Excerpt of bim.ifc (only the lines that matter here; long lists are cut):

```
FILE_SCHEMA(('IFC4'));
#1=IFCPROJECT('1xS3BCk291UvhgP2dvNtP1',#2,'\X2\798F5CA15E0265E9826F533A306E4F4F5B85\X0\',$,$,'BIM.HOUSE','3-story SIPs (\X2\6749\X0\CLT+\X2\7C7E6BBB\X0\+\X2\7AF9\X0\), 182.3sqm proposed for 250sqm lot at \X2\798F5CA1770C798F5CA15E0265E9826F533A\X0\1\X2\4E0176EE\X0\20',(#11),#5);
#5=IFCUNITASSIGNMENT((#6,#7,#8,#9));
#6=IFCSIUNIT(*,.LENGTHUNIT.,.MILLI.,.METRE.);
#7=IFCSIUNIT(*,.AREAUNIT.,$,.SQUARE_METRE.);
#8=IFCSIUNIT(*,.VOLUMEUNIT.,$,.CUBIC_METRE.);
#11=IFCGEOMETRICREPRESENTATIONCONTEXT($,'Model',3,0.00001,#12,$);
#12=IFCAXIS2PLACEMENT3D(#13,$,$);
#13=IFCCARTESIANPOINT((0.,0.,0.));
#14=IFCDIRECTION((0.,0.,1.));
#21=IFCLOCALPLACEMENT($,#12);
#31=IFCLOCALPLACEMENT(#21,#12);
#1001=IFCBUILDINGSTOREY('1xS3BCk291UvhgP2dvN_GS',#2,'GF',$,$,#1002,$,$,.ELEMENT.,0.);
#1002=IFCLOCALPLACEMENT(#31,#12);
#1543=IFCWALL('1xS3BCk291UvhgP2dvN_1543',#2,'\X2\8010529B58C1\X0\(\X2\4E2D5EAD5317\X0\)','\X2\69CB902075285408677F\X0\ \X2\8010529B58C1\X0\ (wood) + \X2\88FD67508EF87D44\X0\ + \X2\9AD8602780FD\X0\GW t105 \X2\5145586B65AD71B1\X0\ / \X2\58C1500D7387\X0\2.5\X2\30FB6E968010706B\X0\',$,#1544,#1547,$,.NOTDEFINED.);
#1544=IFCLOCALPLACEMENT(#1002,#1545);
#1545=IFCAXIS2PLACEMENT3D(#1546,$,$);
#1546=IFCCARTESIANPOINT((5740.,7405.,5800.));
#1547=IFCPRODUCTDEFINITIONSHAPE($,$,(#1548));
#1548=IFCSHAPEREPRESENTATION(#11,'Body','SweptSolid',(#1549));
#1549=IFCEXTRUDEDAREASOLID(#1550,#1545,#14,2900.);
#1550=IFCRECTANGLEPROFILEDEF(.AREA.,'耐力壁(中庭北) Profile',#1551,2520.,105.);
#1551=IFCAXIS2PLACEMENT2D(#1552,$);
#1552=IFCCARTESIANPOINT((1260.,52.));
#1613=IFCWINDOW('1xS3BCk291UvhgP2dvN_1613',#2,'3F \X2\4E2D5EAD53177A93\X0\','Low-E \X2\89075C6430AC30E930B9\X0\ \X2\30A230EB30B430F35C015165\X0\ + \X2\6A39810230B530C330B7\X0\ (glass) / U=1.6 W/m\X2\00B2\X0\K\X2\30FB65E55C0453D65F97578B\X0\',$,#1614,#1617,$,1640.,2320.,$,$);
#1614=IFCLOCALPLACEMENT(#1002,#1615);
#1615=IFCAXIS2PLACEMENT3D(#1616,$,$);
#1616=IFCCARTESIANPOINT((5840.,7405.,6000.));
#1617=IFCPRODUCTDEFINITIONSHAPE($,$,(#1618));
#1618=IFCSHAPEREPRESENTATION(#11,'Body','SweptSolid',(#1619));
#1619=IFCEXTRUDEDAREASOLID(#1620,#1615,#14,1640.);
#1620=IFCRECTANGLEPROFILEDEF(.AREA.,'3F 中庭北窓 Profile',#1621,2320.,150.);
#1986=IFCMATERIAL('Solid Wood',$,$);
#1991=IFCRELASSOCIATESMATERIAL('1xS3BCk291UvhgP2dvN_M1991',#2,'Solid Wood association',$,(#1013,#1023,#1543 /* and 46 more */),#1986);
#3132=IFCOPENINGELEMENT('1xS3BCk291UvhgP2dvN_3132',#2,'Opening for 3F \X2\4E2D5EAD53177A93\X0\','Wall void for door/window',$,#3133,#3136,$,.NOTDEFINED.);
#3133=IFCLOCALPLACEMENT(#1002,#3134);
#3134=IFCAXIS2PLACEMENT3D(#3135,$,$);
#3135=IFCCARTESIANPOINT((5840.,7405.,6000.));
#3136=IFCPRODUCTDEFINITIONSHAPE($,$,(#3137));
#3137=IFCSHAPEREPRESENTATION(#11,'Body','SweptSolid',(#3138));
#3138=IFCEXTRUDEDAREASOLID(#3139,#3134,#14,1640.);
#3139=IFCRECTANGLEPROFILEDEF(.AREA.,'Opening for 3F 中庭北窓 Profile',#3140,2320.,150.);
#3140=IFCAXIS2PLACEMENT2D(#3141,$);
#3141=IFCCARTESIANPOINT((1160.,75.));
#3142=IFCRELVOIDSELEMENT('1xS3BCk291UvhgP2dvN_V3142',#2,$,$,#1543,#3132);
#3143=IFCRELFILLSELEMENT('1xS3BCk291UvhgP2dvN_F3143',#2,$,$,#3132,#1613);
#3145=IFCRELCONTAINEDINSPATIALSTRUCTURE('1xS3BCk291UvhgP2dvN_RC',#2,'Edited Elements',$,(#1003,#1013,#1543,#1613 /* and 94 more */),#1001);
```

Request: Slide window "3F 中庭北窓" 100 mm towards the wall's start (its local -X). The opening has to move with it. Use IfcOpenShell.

```python
import ifcopenshell
import ifcopenshell.api.geometry
import ifcopenshell.util.placement

model = ifcopenshell.open("bim.ifc")

window = model.by_id(1613)
opening = window.FillsVoids[0].RelatingOpeningElement
wall = opening.VoidsElements[0].RelatingBuildingElement

wall_matrix = ifcopenshell.util.placement.get_local_placement(wall.ObjectPlacement)
shift = wall_matrix[:3, 0] * -100.0
before = ifcopenshell.util.placement.get_local_placement(window.ObjectPlacement)[:3, 3].copy()

# The window is not placed relative to its opening, so move both.
for product in (opening, window):
    matrix = ifcopenshell.util.placement.get_local_placement(product.ObjectPlacement)
    matrix[:3, 3] += shift
    ifcopenshell.api.geometry.edit_object_placement(model, product=product, matrix=matrix, is_si=False)

after = ifcopenshell.util.placement.get_local_placement(window.ObjectPlacement)[:3, 3]
print("window moved by", (after - before).round(3) + 0.0)

model.write("bim_edited.ifc")
```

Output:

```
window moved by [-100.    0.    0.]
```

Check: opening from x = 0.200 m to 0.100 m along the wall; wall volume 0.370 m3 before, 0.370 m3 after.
